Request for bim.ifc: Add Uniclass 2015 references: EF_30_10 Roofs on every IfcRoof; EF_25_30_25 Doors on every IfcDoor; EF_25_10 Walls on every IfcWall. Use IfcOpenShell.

First a look at what the model holds.

```python
import ifcopenshell

model = ifcopenshell.open("bim.ifc")
print(model.schema)
print("classifications:", [c.Name for c in model.by_type("IfcClassification")])
for ifc_class in ("IfcDoor", "IfcRoof", "IfcStair", "IfcWall", "IfcWindow"):
    print(ifc_class, len(model.by_type(ifc_class)))
```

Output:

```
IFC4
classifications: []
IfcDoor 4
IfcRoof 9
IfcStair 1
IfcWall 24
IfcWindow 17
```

```python
import ifcopenshell
import ifcopenshell.api.classification

model = ifcopenshell.open("bim.ifc")

system = ifcopenshell.api.classification.add_classification(model, classification="Uniclass 2015")

codes = {
    "IfcRoof": ("EF_30_10", "Roofs"),
    "IfcDoor": ("EF_25_30_25", "Doors"),
    "IfcWall": ("EF_25_10", "Walls"),
}
for ifc_class, (code, name) in codes.items():
    products = model.by_type(ifc_class)
    ifcopenshell.api.classification.add_reference(
        model, products=products, classification=system, identification=code, name=name
    )
    print(code, len(products))

model.write("bim_rev.ifc")
```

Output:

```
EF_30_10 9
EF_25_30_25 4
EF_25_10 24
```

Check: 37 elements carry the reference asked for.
